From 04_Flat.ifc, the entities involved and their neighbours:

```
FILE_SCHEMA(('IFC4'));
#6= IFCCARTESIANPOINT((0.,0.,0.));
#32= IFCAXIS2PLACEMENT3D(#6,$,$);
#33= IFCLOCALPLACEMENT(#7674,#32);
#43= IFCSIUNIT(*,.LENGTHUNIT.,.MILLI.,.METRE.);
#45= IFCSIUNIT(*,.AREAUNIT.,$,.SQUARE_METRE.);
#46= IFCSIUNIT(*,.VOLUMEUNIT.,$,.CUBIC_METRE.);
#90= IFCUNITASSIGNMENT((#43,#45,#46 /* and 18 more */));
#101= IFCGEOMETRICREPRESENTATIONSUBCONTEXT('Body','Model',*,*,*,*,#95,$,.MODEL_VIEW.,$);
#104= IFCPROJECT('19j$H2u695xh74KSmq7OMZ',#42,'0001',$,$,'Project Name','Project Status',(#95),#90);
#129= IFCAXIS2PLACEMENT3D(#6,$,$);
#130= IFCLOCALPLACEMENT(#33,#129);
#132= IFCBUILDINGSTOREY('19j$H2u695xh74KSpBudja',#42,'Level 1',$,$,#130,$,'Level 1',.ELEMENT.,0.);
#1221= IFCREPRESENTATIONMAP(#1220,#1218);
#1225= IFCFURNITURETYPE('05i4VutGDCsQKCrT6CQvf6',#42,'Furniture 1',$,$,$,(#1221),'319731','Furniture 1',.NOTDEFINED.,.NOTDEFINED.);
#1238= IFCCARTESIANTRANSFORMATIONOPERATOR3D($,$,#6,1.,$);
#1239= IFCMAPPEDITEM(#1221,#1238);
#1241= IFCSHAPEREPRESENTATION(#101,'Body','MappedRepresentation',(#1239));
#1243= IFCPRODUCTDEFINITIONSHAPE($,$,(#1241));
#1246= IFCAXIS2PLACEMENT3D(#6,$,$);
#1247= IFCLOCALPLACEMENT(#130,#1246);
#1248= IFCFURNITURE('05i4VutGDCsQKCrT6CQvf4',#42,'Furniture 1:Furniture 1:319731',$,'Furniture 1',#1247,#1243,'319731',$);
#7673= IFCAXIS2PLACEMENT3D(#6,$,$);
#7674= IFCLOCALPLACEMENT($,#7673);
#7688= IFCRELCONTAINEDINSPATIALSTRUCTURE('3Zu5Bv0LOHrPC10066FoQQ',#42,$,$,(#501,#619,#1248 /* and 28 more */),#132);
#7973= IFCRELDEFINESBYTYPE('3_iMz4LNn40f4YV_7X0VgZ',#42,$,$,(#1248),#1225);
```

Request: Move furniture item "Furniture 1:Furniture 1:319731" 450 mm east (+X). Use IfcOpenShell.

```python
import ifcopenshell
import ifcopenshell.api.geometry
import ifcopenshell.util.placement
import ifcopenshell.util.unit

model = ifcopenshell.open("04_Flat.ifc")
unit_scale = ifcopenshell.util.unit.calculate_unit_scale(model)

item = model.by_guid("05i4VutGDCsQKCrT6CQvf4")
matrix = ifcopenshell.util.placement.get_local_placement(item.ObjectPlacement)
matrix[0, 3] += 0.45 / unit_scale
ifcopenshell.api.geometry.edit_object_placement(model, product=item, matrix=matrix, is_si=False)

print(ifcopenshell.util.placement.get_local_placement(item.ObjectPlacement).round(3) + 0.0)

model.write("04_Flat_updated.ifc")
```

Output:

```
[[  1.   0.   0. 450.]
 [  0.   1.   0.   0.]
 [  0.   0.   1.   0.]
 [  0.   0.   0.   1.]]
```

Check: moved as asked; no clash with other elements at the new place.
